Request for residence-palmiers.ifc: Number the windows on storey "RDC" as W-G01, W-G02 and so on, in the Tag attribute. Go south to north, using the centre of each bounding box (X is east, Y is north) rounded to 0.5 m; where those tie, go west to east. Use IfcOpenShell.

First a look at what the model holds.

```python
import ifcopenshell
import ifcopenshell.util.element
import ifcopenshell.util.placement

model = ifcopenshell.open("residence-palmiers.ifc")
print(model.schema)
storey = next(s for s in model.by_type("IfcBuildingStorey") if s.Name == "RDC")
windows = [e for e in ifcopenshell.util.element.get_decomposition(storey) if e.is_a("IfcWindow")]
for e in sorted(windows, key=lambda e: e.id()):
    origin = ifcopenshell.util.placement.get_local_placement(e.ObjectPlacement)[:3, 3]
    print(e.id(), e.Tag, e.Name, origin.round(2) + 0.0, sep=" | ")
```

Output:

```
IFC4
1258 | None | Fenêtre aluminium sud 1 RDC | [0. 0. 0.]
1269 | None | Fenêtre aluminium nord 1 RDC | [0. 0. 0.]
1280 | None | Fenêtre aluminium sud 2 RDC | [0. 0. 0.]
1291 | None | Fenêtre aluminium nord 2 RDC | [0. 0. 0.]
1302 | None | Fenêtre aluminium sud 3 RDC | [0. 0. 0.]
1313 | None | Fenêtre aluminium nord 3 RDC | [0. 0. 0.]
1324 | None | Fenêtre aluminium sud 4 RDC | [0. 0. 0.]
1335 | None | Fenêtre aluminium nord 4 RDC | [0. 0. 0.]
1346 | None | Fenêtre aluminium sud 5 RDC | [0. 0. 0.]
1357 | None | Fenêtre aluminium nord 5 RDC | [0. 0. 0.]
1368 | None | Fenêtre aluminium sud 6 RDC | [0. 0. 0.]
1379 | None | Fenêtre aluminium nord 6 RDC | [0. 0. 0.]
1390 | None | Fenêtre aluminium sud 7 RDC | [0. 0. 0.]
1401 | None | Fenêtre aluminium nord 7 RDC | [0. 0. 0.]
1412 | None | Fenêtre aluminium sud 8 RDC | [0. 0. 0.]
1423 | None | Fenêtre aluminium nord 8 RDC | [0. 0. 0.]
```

```python
import ifcopenshell
import ifcopenshell.geom
import ifcopenshell.util.element
import ifcopenshell.util.shape

model = ifcopenshell.open("residence-palmiers.ifc")
settings = ifcopenshell.geom.settings()
settings.set("use-world-coords", True)


def centre(element):
    shape = ifcopenshell.geom.create_shape(settings, element)
    return ifcopenshell.util.shape.get_bbox_centroid(shape.geometry)


storey = next(s for s in model.by_type("IfcBuildingStorey") if s.Name == "RDC")
windows = [e for e in ifcopenshell.util.element.get_decomposition(storey) if e.is_a("IfcWindow")]

# Insertion points can sit at a corner or the storey origin, so sort by the geometry (in metres).
centres = {e: centre(e) for e in windows}
windows.sort(key=lambda e: (round(centres[e][1] / 0.5), centres[e][0]))

for i, e in enumerate(windows, start=1):
    number = f"W-G{i:02d}"
    e.Tag = number
    print(e.id(), number)

model.write("residence-palmiers_edited.ifc")
```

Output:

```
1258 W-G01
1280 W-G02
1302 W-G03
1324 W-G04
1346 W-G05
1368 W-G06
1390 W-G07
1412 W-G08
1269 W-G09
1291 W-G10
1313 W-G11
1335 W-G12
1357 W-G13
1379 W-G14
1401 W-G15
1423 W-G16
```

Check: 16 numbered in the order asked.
